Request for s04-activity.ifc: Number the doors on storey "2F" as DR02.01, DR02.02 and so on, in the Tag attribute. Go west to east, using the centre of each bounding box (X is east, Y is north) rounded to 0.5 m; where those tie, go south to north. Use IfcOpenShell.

First a look at what the model holds.

```python
import ifcopenshell
import ifcopenshell.util.element
import ifcopenshell.util.placement

model = ifcopenshell.open("s04-activity.ifc")
print(model.schema)
storey = next(s for s in model.by_type("IfcBuildingStorey") if s.Name == "2F")
doors = [e for e in ifcopenshell.util.element.get_decomposition(storey) if e.is_a("IfcDoor")]
for e in sorted(doors, key=lambda e: e.id()):
    origin = ifcopenshell.util.placement.get_local_placement(e.ObjectPlacement)[:3, 3]
    print(e.id(), e.Tag, e.Name, origin.round(2) + 0.0, sep=" | ")
```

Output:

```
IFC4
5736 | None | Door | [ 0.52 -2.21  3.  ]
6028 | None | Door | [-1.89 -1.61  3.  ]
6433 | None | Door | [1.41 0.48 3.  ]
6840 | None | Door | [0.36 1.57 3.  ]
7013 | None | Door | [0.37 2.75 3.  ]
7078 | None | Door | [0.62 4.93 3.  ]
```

```python
import ifcopenshell
import ifcopenshell.geom
import ifcopenshell.util.element
import ifcopenshell.util.shape

model = ifcopenshell.open("s04-activity.ifc")
settings = ifcopenshell.geom.settings()
settings.set("use-world-coords", True)


def centre(element):
    shape = ifcopenshell.geom.create_shape(settings, element)
    return ifcopenshell.util.shape.get_bbox_centroid(shape.geometry)


storey = next(s for s in model.by_type("IfcBuildingStorey") if s.Name == "2F")
doors = [e for e in ifcopenshell.util.element.get_decomposition(storey) if e.is_a("IfcDoor")]

# Insertion points can sit at a corner or the storey origin, so sort by the geometry (in metres).
centres = {e: centre(e) for e in doors}
doors.sort(key=lambda e: (round(centres[e][0] / 0.5), centres[e][1]))

for i, e in enumerate(doors, start=1):
    number = f"DR02.{i:02d}"
    e.Tag = number
    print(e.id(), number)

model.write("s04-activity_rev.ifc")
```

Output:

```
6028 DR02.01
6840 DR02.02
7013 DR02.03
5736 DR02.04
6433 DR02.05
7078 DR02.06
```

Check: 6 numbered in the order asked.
